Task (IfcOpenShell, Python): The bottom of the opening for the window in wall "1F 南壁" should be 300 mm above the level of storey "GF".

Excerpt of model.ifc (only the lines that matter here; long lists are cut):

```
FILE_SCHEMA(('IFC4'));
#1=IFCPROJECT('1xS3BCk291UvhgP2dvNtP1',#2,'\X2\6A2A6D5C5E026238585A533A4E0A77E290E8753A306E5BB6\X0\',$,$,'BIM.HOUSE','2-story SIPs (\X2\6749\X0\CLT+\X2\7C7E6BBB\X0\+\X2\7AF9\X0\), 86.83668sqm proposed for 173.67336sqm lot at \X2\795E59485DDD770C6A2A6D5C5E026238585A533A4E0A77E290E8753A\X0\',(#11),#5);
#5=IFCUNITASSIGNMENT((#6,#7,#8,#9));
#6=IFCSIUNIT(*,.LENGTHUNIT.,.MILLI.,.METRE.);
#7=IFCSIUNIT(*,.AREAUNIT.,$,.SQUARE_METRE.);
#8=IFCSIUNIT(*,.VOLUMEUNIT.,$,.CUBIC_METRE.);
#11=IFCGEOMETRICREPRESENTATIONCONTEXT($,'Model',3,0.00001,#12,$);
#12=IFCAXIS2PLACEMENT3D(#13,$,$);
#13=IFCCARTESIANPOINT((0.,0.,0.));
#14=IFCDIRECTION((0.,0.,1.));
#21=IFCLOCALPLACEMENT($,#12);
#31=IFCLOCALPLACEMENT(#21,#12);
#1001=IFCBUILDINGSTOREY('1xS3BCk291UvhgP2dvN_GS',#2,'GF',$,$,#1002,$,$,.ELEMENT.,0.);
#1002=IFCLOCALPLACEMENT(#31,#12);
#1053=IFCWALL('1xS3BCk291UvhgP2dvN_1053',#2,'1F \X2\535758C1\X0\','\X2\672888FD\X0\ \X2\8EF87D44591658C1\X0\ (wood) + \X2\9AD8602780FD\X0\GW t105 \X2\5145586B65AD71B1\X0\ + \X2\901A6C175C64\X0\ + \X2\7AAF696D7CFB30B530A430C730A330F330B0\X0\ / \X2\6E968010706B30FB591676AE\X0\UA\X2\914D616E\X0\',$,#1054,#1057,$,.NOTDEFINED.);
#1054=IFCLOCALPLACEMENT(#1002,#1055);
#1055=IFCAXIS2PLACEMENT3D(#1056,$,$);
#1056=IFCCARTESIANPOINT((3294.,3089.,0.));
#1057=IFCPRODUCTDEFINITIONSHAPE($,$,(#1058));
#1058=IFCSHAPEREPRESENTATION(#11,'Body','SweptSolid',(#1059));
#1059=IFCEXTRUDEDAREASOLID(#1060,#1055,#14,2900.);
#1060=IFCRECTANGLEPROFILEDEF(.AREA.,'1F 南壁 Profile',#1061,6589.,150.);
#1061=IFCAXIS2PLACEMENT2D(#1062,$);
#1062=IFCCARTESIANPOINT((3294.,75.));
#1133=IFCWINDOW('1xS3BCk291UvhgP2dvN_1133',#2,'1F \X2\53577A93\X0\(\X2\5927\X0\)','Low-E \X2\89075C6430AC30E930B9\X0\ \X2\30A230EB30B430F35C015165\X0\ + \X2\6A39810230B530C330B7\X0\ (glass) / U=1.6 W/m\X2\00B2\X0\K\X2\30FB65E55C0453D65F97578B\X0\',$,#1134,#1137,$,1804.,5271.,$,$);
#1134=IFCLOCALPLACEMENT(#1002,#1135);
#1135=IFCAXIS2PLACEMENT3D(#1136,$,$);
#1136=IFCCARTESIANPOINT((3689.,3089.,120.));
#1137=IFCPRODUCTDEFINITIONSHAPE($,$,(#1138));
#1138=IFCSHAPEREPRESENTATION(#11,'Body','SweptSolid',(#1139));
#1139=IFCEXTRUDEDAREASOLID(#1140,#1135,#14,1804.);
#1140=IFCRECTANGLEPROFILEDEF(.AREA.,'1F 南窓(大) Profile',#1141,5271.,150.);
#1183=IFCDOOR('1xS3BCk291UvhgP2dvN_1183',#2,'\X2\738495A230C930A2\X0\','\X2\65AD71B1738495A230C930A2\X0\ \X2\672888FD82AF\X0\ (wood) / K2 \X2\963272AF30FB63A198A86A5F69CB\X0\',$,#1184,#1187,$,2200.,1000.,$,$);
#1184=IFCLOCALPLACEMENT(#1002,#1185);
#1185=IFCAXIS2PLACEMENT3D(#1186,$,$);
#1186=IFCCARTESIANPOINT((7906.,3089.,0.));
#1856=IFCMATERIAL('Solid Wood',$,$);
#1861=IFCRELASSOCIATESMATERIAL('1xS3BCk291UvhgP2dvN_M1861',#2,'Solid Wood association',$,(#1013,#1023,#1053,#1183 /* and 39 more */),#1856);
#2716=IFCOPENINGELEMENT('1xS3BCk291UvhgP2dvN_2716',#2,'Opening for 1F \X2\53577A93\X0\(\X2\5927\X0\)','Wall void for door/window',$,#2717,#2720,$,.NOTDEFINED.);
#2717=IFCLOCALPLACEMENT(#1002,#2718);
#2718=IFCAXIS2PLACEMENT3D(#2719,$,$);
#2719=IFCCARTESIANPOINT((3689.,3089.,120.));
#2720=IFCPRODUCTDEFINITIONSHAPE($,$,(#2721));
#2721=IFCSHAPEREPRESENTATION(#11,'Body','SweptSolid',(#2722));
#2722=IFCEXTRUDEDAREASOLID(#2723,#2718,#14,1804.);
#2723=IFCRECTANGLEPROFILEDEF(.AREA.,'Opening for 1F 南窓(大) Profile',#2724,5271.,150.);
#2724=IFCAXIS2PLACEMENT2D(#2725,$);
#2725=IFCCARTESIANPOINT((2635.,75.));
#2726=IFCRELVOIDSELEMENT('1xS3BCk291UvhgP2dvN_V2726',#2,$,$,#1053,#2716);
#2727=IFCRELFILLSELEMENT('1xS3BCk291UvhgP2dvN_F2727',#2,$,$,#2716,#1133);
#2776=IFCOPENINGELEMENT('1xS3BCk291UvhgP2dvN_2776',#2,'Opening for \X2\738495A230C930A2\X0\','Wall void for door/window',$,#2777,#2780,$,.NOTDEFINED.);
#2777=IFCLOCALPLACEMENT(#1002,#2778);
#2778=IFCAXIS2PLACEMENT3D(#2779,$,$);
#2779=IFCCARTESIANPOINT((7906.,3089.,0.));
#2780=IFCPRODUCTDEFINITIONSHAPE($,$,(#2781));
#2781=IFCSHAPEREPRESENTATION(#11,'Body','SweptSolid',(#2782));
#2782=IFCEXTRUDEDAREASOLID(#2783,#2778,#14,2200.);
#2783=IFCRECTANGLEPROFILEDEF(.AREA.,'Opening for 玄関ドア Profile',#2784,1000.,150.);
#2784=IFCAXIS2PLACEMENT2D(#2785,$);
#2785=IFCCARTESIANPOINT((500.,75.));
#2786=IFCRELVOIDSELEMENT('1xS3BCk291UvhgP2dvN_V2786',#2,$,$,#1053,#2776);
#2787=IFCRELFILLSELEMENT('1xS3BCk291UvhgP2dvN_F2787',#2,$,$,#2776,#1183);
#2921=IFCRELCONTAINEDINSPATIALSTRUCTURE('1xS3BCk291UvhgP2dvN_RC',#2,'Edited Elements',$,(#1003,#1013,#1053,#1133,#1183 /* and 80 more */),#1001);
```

```python
import numpy as np
import ifcopenshell
import ifcopenshell.api.geometry
import ifcopenshell.geom
import ifcopenshell.util.element
import ifcopenshell.util.placement
import ifcopenshell.util.shape
import ifcopenshell.util.unit

model = ifcopenshell.open("model.ifc")
unit_scale = ifcopenshell.util.unit.calculate_unit_scale(model)

window = model.by_guid("1xS3BCk291UvhgP2dvN_1133")
opening = window.FillsVoids[0].RelatingOpeningElement
storey = ifcopenshell.util.element.get_container(window, ifc_class="IfcBuildingStorey")
level = ifcopenshell.util.placement.get_local_placement(storey.ObjectPlacement)[2, 3]

# The opening's origin need not be at the sill, so measure its lowest point.
shape = ifcopenshell.geom.create_shape(ifcopenshell.geom.settings(), opening)
bottom = ifcopenshell.util.shape.get_shape_bottom_elevation(shape, shape.geometry) / unit_scale
dz = level + 0.3 / unit_scale - bottom

shift = np.array([0.0, 0.0, dz])
# The window is not placed relative to its opening, so move both.
for product in (opening, window):
    matrix = ifcopenshell.util.placement.get_local_placement(product.ObjectPlacement)
    matrix[:3, 3] += shift
    ifcopenshell.api.geometry.edit_object_placement(model, product=product, matrix=matrix, is_si=False)

print(f"moved by {dz * unit_scale:+.3f} m")

model.write("model_v2.ifc")
```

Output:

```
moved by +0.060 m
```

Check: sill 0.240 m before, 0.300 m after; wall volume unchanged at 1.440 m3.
